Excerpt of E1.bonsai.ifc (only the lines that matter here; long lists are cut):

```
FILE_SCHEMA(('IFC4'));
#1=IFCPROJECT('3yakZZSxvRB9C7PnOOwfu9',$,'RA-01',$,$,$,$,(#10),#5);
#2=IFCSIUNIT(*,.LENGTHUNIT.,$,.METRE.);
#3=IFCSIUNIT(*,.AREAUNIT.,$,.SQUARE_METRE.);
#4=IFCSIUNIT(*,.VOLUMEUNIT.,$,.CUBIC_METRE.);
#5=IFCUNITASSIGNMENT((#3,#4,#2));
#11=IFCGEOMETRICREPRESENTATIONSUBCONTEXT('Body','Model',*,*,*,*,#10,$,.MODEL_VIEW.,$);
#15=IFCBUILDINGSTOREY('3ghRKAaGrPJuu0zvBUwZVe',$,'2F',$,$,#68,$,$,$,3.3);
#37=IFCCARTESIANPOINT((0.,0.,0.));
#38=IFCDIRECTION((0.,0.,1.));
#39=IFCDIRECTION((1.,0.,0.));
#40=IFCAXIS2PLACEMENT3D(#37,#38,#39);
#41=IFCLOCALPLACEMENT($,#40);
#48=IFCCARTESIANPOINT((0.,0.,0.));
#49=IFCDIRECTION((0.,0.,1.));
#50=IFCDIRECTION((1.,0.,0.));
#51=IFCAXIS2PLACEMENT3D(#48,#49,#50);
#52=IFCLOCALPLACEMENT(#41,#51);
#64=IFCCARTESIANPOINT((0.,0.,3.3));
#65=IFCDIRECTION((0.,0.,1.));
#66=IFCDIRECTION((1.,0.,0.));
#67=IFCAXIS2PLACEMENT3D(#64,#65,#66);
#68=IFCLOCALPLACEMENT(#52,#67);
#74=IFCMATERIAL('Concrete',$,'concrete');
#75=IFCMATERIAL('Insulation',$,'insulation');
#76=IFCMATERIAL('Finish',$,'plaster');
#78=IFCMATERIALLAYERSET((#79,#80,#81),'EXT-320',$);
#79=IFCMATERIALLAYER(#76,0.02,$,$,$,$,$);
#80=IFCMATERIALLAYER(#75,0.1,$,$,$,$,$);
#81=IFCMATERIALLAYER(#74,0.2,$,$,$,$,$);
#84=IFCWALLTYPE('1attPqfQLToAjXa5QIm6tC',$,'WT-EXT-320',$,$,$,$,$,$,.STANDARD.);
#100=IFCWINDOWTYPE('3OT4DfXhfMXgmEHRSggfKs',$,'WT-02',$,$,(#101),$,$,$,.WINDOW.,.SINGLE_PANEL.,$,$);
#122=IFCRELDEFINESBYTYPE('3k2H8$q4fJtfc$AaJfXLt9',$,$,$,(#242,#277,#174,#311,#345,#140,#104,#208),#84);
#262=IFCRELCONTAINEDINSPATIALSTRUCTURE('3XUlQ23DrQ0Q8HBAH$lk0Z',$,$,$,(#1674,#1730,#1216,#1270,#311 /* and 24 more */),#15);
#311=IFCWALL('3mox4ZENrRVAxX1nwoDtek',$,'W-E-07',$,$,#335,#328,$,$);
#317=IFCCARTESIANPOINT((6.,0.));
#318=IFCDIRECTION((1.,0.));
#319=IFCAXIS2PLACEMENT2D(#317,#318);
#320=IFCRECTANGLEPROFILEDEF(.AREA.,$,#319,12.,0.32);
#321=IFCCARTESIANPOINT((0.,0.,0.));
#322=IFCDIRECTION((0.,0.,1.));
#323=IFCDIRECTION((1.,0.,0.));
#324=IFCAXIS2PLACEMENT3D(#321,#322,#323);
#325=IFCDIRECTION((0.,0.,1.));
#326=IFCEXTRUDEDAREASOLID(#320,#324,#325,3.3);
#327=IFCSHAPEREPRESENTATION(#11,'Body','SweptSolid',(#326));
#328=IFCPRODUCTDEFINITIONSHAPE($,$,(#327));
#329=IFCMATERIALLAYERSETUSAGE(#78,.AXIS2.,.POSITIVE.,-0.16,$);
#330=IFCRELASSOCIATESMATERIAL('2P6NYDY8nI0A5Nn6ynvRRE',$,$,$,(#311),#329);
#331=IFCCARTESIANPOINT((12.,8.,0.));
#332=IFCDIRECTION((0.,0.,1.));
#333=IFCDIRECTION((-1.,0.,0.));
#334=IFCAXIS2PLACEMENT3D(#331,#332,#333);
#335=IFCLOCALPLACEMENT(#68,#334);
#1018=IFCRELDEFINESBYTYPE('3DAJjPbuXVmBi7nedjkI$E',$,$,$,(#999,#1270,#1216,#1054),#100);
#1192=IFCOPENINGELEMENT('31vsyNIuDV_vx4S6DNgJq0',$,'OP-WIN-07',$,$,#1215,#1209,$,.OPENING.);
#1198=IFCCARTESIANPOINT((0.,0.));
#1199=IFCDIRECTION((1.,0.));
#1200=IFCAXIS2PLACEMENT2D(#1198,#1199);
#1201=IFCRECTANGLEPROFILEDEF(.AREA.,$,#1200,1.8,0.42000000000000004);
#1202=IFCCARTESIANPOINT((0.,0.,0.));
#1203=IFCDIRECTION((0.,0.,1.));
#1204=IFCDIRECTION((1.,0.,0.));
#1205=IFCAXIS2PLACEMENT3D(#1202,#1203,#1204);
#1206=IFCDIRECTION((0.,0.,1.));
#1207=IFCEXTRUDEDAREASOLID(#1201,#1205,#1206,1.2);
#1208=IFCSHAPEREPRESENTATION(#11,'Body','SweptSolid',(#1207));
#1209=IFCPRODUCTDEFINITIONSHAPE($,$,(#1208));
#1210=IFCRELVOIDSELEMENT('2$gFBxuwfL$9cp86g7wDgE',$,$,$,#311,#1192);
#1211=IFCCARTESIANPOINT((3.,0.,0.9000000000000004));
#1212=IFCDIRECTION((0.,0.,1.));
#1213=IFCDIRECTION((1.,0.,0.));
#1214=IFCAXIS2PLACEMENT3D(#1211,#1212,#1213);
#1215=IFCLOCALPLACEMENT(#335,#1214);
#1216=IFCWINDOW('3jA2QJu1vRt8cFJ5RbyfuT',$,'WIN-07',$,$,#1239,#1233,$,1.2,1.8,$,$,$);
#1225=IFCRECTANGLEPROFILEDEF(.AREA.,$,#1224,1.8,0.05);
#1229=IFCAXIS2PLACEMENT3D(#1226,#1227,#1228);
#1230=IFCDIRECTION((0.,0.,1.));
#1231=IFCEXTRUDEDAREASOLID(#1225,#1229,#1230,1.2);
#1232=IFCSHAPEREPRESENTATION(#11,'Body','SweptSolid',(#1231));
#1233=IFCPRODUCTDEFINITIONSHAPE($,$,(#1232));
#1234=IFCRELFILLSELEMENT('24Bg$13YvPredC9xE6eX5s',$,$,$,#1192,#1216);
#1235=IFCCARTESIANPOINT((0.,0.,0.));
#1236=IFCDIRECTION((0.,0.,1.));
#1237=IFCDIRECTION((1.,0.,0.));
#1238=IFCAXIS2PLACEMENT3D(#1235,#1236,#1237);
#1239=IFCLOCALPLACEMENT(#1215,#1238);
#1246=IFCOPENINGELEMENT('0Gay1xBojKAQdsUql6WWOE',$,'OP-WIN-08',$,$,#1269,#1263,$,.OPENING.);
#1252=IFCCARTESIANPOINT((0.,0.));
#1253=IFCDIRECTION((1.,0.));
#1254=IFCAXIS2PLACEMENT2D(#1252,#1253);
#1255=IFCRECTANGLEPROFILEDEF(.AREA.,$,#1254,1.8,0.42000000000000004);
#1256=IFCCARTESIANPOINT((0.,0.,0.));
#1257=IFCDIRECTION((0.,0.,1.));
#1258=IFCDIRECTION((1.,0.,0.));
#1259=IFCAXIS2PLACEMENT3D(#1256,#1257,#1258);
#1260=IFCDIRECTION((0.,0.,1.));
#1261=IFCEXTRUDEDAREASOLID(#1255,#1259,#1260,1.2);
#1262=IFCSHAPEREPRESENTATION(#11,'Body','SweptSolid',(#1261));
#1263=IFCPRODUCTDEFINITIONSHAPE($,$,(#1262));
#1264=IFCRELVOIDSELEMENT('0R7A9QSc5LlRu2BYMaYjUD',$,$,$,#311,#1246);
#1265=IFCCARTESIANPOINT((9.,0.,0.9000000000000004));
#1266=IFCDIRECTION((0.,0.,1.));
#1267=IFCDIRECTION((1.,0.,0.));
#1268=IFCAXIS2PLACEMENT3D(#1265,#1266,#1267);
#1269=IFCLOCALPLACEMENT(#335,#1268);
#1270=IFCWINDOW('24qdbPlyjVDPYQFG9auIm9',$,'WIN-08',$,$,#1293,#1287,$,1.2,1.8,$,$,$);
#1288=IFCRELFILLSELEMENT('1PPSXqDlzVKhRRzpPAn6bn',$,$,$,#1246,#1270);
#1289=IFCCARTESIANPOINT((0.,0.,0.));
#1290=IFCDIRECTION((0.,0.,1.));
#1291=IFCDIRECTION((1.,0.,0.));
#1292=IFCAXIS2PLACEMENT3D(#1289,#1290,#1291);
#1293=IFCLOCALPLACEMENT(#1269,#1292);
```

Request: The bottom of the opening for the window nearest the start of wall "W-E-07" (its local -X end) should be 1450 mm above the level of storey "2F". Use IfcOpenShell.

```python
import numpy as np
import ifcopenshell
import ifcopenshell.api.geometry
import ifcopenshell.geom
import ifcopenshell.util.element
import ifcopenshell.util.placement
import ifcopenshell.util.shape
import ifcopenshell.util.unit

model = ifcopenshell.open("E1.bonsai.ifc")
unit_scale = ifcopenshell.util.unit.calculate_unit_scale(model)

window = model.by_id(1216)
opening = window.FillsVoids[0].RelatingOpeningElement
storey = ifcopenshell.util.element.get_container(window, ifc_class="IfcBuildingStorey")
level = ifcopenshell.util.placement.get_local_placement(storey.ObjectPlacement)[2, 3]

# The opening's origin need not be at the sill, so measure its lowest point.
shape = ifcopenshell.geom.create_shape(ifcopenshell.geom.settings(), opening)
bottom = ifcopenshell.util.shape.get_shape_bottom_elevation(shape, shape.geometry) / unit_scale
dz = level + 1.45 - bottom

shift = np.array([0.0, 0.0, dz])
# The window is placed relative to its opening, so it follows when the opening moves.
matrix = ifcopenshell.util.placement.get_local_placement(opening.ObjectPlacement)
matrix[:3, 3] += shift
ifcopenshell.api.geometry.edit_object_placement(
    model, product=opening, matrix=matrix, is_si=False, should_transform_children=True
)

print(f"moved by {dz * unit_scale:+.3f} m")

model.write("E1.bonsai_rev.ifc")
```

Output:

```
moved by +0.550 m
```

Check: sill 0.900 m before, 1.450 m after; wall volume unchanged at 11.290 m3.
